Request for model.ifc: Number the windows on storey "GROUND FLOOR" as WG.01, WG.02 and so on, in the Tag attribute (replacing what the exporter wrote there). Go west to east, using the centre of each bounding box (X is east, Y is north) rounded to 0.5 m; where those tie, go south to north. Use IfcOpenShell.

First a look at what the model holds.

```python
import ifcopenshell
import ifcopenshell.util.element
import ifcopenshell.util.placement

model = ifcopenshell.open("model.ifc")
print(model.schema)
storey = next(s for s in model.by_type("IfcBuildingStorey") if s.Name == "GROUND FLOOR")
windows = [e for e in ifcopenshell.util.element.get_decomposition(storey) if e.is_a("IfcWindow")]
for e in sorted(windows, key=lambda e: e.id()):
    origin = ifcopenshell.util.placement.get_local_placement(e.ObjectPlacement)[:3, 3]
    print(e.id(), e.Tag, e.Name, origin.round(2) + 0.0, sep=" | ")
```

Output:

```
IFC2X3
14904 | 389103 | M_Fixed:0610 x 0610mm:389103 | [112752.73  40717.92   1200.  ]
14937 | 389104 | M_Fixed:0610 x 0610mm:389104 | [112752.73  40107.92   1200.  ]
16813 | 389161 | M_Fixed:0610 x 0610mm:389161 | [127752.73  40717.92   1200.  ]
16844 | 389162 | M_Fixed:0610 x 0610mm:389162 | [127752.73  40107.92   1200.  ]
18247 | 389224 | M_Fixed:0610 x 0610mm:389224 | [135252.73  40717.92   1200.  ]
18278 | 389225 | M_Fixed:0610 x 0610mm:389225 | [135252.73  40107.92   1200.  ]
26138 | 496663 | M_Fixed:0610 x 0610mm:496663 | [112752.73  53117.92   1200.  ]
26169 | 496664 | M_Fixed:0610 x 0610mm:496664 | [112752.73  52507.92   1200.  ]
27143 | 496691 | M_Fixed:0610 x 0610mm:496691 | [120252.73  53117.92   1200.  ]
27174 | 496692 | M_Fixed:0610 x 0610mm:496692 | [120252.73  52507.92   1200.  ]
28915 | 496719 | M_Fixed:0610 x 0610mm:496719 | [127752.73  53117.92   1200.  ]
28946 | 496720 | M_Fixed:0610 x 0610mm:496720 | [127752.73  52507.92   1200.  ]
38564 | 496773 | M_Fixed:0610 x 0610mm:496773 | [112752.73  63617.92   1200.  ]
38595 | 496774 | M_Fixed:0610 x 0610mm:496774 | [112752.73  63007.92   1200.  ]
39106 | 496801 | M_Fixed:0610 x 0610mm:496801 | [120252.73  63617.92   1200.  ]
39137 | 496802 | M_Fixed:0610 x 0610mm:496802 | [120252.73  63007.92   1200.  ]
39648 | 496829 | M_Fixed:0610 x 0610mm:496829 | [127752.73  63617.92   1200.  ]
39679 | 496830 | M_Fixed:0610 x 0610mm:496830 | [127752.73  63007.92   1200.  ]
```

```python
import ifcopenshell
import ifcopenshell.geom
import ifcopenshell.util.element
import ifcopenshell.util.shape

model = ifcopenshell.open("model.ifc")
settings = ifcopenshell.geom.settings()
settings.set("use-world-coords", True)


def centre(element):
    shape = ifcopenshell.geom.create_shape(settings, element)
    return ifcopenshell.util.shape.get_bbox_centroid(shape.geometry)


storey = next(s for s in model.by_type("IfcBuildingStorey") if s.Name == "GROUND FLOOR")
windows = [e for e in ifcopenshell.util.element.get_decomposition(storey) if e.is_a("IfcWindow")]

# Insertion points can sit at a corner or the storey origin, so sort by the geometry (in metres).
centres = {e: centre(e) for e in windows}
windows.sort(key=lambda e: (round(centres[e][0] / 0.5), centres[e][1]))

for i, e in enumerate(windows, start=1):
    number = f"WG.{i:02d}"
    e.Tag = number
    print(e.id(), number)

model.write("model_edited.ifc")
```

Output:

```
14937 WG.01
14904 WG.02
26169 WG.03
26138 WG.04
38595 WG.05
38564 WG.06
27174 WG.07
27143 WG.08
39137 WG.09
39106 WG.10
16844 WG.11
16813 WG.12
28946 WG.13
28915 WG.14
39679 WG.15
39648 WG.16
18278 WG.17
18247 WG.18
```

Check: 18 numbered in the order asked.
